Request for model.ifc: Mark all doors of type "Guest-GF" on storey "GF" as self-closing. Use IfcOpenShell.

First a look at what the model holds.

```python
import ifcopenshell
import ifcopenshell.util.element

model = ifcopenshell.open("model.ifc")
print(model.schema)
storey = next(s for s in model.by_type("IfcBuildingStorey") if s.Name == "GF")
doors = [e for e in ifcopenshell.util.element.get_decomposition(storey) if e.is_a("IfcDoor")]
seen = {}
for e in doors:
    element_type = ifcopenshell.util.element.get_type(e)
    key = (element_type.Name if element_type != e and element_type else None, ifcopenshell.util.element.get_pset(e, "Pset_DoorCommon", "SelfClosing"))
    seen[key] = seen.get(key, 0) + 1
for (name, value), count in sorted(seen.items(), key=str):
    print(count, "x", name, "|", value)
```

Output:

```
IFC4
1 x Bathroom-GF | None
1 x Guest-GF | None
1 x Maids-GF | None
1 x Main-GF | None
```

```python
import ifcopenshell
import ifcopenshell.api.pset
import ifcopenshell.util.element

model = ifcopenshell.open("model.ifc")

storey = next(s for s in model.by_type("IfcBuildingStorey") if s.Name == "GF")
doors = [e for e in ifcopenshell.util.element.get_decomposition(storey) if e.is_a("IfcDoor")]

count = 0
for e in doors:
    element_type = ifcopenshell.util.element.get_type(e)
    if element_type in (None, e) or element_type.Name != "Guest-GF":
        continue
    # add_pset returns the element's existing set when there is one.
    pset = ifcopenshell.api.pset.add_pset(model, product=e, name="Pset_DoorCommon")
    ifcopenshell.api.pset.edit_pset(model, pset=pset, properties={"SelfClosing": True})
    count += 1

print(count, "doors updated")

model.write("model_updated.ifc")
```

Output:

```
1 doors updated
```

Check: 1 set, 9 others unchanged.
